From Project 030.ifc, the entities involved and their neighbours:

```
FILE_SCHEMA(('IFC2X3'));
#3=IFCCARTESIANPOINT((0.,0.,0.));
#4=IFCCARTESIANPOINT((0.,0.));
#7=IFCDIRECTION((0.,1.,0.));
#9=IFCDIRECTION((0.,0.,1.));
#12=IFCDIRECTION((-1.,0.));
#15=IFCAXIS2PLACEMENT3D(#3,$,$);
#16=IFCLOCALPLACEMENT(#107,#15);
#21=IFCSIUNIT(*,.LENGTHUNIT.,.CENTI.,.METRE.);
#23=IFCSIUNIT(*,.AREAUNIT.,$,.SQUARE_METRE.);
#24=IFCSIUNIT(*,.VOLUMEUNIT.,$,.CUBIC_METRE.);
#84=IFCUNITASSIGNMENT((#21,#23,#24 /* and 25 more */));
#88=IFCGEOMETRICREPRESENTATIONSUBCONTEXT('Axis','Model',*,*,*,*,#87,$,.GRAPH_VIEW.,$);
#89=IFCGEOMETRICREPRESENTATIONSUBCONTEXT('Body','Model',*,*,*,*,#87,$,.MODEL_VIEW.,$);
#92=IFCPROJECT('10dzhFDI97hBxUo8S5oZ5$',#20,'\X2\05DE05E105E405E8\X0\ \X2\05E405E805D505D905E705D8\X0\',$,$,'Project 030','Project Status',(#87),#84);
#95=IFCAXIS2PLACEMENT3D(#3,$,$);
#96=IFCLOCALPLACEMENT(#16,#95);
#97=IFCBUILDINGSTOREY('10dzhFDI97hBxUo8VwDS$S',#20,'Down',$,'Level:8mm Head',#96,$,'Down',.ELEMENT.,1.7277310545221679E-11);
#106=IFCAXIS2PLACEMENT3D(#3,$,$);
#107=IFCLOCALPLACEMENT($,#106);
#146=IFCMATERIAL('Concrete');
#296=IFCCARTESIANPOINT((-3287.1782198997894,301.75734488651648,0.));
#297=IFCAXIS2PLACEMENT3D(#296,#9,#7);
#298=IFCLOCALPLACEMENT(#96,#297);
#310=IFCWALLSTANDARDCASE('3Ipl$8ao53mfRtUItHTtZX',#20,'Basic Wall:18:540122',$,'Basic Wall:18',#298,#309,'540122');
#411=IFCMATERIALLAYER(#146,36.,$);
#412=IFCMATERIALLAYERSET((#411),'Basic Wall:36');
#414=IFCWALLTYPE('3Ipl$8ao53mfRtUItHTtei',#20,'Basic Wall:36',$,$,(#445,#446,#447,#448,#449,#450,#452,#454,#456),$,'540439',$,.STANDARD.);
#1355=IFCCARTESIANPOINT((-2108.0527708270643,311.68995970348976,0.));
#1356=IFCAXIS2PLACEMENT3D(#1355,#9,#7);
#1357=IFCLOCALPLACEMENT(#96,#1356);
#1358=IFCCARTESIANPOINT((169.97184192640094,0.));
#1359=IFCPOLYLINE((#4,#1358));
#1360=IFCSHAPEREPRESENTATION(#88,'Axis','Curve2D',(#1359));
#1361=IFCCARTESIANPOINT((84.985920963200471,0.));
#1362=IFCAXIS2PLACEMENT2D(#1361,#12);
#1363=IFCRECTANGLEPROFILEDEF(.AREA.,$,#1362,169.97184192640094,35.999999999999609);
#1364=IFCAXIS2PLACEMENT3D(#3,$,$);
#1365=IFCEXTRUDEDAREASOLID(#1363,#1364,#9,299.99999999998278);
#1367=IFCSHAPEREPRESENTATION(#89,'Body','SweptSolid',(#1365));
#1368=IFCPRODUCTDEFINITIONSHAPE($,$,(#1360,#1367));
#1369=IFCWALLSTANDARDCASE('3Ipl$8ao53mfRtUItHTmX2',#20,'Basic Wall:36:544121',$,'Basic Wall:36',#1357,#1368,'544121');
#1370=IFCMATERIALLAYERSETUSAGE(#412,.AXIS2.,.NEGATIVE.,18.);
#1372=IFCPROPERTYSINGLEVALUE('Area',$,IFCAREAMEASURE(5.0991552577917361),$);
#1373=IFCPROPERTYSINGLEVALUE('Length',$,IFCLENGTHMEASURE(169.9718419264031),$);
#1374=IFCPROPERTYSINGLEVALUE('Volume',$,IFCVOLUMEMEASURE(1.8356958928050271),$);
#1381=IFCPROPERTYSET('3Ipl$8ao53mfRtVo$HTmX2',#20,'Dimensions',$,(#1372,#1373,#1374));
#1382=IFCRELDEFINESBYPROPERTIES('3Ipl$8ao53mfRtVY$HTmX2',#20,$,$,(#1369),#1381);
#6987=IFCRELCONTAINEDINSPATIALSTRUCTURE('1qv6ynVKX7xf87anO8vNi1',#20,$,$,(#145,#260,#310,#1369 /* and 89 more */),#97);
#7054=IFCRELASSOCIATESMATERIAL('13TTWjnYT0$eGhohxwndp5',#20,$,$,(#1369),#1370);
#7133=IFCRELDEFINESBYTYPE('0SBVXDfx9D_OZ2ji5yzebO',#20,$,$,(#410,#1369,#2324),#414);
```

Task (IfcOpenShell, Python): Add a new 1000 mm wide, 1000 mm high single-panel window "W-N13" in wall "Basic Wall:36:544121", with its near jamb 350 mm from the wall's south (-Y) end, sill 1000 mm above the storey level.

```python
import numpy as np
import ifcopenshell
import ifcopenshell.api.feature
import ifcopenshell.api.geometry
import ifcopenshell.api.pset
import ifcopenshell.api.root
import ifcopenshell.api.spatial
import ifcopenshell.api.type
import ifcopenshell.geom
import ifcopenshell.util.element
import ifcopenshell.util.placement
import ifcopenshell.util.representation
import ifcopenshell.util.shape
import ifcopenshell.util.unit

model = ifcopenshell.open("Project 030.ifc")
unit_scale = ifcopenshell.util.unit.calculate_unit_scale(model)
area_scale = ifcopenshell.util.unit.calculate_unit_scale(model, "AREAUNIT")
volume_scale = ifcopenshell.util.unit.calculate_unit_scale(model, "VOLUMEUNIT")
settings = ifcopenshell.geom.settings()


def volume(element):
    """Net volume in cubic metres, openings subtracted."""
    shape = ifcopenshell.geom.create_shape(settings, element)
    return ifcopenshell.util.shape.get_volume(shape.geometry)


wall = model.by_id(1369)
storey = ifcopenshell.util.element.get_container(wall, ifc_class="IfcBuildingStorey")
context = ifcopenshell.util.representation.get_context(model, "Model", "Body", "MODEL_VIEW")
before = volume(wall)

width, height, from_end, sill = 1, 1, 0.35, 1  # metres

# The wall runs along its own X axis, and the end named is its -X end.
wall_shape = ifcopenshell.geom.create_shape(settings, wall)
x, y, z = ifcopenshell.util.shape.get_vertices(wall_shape.geometry).T
start = x.min() + from_end
face, thickness = float(y.min()), float(y.max() - y.min())
wall_matrix = ifcopenshell.util.placement.get_local_placement(wall.ObjectPlacement)
level = ifcopenshell.util.placement.get_local_placement(storey.ObjectPlacement)[2, 3]


def in_wall(x, y):
    """Placement at x, y metres in the wall's axes, at sill height."""
    matrix = wall_matrix.copy()
    matrix[:, 3] = wall_matrix @ np.array([x / unit_scale, y / unit_scale, 0.0, 1.0])
    matrix[2, 3] = level + sill / unit_scale
    return matrix


# Opening: a box that overshoots both wall faces by 50 mm.
opening = ifcopenshell.api.root.create_entity(model, ifc_class="IfcOpeningElement")
box = ifcopenshell.api.geometry.add_wall_representation(
    model, context=context, length=width, height=height, thickness=thickness + 0.1
)
ifcopenshell.api.geometry.assign_representation(model, product=opening, representation=box)
ifcopenshell.api.geometry.edit_object_placement(model, product=opening, matrix=in_wall(start, face - 0.05), is_si=False)
ifcopenshell.api.feature.add_feature(model, feature=opening, element=wall)

window = ifcopenshell.api.root.create_entity(model, ifc_class="IfcWindow", name="W-N13")
window.OverallWidth, window.OverallHeight = width / unit_scale, height / unit_scale
body = ifcopenshell.api.geometry.add_window_representation(
    model,
    context=context,
    overall_width=window.OverallWidth,
    overall_height=window.OverallHeight,
    partition_type="SINGLE_PANEL",
)
ifcopenshell.api.geometry.assign_representation(model, product=window, representation=body)
ifcopenshell.api.spatial.assign_container(model, products=[window], relating_structure=storey)
fills = ifcopenshell.api.feature.add_filling(model, opening=opening, element=window)
fills.OwnerHistory = window.OwnerHistory  # required in IFC2X3

# IFC2X3 keeps the operation on the window style.
style = ifcopenshell.api.root.create_entity(model, ifc_class="IfcWindowStyle", name="W-N13")
style.OperationType, style.ConstructionType = "SINGLE_PANEL", "NOTDEFINED"
style.ParameterTakesPrecedence = style.Sizeable = False
ifcopenshell.api.type.assign_type(model, related_objects=[window], relating_type=style)

# Centre the window in the wall's thickness.
ifcopenshell.api.geometry.edit_object_placement(model, product=window, matrix=in_wall(start, face), is_si=False)
window_shape = ifcopenshell.geom.create_shape(settings, window)
depth = ifcopenshell.util.shape.get_vertices(window_shape.geometry)[:, 1]
offset = face + thickness / 2 - (depth.min() + depth.max()) / 2
ifcopenshell.api.geometry.edit_object_placement(model, product=window, matrix=in_wall(start, offset), is_si=False)

after = volume(wall)

# Update the wall's stored quantities.
pset = model.by_id(ifcopenshell.util.element.get_pset(wall, "Dimensions", should_inherit=False)["id"])
ifcopenshell.api.pset.edit_pset(model, pset=pset, properties={
    "Area": model.create_entity("IfcAreaMeasure", after / thickness / area_scale),
    "Volume": model.create_entity("IfcVolumeMeasure", after / volume_scale),
})

print(f"wall volume {before:.3f} -> {after:.3f} m3")

model.write("Project 030_v2.ifc")
```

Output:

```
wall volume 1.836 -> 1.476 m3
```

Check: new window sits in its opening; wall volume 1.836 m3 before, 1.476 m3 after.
